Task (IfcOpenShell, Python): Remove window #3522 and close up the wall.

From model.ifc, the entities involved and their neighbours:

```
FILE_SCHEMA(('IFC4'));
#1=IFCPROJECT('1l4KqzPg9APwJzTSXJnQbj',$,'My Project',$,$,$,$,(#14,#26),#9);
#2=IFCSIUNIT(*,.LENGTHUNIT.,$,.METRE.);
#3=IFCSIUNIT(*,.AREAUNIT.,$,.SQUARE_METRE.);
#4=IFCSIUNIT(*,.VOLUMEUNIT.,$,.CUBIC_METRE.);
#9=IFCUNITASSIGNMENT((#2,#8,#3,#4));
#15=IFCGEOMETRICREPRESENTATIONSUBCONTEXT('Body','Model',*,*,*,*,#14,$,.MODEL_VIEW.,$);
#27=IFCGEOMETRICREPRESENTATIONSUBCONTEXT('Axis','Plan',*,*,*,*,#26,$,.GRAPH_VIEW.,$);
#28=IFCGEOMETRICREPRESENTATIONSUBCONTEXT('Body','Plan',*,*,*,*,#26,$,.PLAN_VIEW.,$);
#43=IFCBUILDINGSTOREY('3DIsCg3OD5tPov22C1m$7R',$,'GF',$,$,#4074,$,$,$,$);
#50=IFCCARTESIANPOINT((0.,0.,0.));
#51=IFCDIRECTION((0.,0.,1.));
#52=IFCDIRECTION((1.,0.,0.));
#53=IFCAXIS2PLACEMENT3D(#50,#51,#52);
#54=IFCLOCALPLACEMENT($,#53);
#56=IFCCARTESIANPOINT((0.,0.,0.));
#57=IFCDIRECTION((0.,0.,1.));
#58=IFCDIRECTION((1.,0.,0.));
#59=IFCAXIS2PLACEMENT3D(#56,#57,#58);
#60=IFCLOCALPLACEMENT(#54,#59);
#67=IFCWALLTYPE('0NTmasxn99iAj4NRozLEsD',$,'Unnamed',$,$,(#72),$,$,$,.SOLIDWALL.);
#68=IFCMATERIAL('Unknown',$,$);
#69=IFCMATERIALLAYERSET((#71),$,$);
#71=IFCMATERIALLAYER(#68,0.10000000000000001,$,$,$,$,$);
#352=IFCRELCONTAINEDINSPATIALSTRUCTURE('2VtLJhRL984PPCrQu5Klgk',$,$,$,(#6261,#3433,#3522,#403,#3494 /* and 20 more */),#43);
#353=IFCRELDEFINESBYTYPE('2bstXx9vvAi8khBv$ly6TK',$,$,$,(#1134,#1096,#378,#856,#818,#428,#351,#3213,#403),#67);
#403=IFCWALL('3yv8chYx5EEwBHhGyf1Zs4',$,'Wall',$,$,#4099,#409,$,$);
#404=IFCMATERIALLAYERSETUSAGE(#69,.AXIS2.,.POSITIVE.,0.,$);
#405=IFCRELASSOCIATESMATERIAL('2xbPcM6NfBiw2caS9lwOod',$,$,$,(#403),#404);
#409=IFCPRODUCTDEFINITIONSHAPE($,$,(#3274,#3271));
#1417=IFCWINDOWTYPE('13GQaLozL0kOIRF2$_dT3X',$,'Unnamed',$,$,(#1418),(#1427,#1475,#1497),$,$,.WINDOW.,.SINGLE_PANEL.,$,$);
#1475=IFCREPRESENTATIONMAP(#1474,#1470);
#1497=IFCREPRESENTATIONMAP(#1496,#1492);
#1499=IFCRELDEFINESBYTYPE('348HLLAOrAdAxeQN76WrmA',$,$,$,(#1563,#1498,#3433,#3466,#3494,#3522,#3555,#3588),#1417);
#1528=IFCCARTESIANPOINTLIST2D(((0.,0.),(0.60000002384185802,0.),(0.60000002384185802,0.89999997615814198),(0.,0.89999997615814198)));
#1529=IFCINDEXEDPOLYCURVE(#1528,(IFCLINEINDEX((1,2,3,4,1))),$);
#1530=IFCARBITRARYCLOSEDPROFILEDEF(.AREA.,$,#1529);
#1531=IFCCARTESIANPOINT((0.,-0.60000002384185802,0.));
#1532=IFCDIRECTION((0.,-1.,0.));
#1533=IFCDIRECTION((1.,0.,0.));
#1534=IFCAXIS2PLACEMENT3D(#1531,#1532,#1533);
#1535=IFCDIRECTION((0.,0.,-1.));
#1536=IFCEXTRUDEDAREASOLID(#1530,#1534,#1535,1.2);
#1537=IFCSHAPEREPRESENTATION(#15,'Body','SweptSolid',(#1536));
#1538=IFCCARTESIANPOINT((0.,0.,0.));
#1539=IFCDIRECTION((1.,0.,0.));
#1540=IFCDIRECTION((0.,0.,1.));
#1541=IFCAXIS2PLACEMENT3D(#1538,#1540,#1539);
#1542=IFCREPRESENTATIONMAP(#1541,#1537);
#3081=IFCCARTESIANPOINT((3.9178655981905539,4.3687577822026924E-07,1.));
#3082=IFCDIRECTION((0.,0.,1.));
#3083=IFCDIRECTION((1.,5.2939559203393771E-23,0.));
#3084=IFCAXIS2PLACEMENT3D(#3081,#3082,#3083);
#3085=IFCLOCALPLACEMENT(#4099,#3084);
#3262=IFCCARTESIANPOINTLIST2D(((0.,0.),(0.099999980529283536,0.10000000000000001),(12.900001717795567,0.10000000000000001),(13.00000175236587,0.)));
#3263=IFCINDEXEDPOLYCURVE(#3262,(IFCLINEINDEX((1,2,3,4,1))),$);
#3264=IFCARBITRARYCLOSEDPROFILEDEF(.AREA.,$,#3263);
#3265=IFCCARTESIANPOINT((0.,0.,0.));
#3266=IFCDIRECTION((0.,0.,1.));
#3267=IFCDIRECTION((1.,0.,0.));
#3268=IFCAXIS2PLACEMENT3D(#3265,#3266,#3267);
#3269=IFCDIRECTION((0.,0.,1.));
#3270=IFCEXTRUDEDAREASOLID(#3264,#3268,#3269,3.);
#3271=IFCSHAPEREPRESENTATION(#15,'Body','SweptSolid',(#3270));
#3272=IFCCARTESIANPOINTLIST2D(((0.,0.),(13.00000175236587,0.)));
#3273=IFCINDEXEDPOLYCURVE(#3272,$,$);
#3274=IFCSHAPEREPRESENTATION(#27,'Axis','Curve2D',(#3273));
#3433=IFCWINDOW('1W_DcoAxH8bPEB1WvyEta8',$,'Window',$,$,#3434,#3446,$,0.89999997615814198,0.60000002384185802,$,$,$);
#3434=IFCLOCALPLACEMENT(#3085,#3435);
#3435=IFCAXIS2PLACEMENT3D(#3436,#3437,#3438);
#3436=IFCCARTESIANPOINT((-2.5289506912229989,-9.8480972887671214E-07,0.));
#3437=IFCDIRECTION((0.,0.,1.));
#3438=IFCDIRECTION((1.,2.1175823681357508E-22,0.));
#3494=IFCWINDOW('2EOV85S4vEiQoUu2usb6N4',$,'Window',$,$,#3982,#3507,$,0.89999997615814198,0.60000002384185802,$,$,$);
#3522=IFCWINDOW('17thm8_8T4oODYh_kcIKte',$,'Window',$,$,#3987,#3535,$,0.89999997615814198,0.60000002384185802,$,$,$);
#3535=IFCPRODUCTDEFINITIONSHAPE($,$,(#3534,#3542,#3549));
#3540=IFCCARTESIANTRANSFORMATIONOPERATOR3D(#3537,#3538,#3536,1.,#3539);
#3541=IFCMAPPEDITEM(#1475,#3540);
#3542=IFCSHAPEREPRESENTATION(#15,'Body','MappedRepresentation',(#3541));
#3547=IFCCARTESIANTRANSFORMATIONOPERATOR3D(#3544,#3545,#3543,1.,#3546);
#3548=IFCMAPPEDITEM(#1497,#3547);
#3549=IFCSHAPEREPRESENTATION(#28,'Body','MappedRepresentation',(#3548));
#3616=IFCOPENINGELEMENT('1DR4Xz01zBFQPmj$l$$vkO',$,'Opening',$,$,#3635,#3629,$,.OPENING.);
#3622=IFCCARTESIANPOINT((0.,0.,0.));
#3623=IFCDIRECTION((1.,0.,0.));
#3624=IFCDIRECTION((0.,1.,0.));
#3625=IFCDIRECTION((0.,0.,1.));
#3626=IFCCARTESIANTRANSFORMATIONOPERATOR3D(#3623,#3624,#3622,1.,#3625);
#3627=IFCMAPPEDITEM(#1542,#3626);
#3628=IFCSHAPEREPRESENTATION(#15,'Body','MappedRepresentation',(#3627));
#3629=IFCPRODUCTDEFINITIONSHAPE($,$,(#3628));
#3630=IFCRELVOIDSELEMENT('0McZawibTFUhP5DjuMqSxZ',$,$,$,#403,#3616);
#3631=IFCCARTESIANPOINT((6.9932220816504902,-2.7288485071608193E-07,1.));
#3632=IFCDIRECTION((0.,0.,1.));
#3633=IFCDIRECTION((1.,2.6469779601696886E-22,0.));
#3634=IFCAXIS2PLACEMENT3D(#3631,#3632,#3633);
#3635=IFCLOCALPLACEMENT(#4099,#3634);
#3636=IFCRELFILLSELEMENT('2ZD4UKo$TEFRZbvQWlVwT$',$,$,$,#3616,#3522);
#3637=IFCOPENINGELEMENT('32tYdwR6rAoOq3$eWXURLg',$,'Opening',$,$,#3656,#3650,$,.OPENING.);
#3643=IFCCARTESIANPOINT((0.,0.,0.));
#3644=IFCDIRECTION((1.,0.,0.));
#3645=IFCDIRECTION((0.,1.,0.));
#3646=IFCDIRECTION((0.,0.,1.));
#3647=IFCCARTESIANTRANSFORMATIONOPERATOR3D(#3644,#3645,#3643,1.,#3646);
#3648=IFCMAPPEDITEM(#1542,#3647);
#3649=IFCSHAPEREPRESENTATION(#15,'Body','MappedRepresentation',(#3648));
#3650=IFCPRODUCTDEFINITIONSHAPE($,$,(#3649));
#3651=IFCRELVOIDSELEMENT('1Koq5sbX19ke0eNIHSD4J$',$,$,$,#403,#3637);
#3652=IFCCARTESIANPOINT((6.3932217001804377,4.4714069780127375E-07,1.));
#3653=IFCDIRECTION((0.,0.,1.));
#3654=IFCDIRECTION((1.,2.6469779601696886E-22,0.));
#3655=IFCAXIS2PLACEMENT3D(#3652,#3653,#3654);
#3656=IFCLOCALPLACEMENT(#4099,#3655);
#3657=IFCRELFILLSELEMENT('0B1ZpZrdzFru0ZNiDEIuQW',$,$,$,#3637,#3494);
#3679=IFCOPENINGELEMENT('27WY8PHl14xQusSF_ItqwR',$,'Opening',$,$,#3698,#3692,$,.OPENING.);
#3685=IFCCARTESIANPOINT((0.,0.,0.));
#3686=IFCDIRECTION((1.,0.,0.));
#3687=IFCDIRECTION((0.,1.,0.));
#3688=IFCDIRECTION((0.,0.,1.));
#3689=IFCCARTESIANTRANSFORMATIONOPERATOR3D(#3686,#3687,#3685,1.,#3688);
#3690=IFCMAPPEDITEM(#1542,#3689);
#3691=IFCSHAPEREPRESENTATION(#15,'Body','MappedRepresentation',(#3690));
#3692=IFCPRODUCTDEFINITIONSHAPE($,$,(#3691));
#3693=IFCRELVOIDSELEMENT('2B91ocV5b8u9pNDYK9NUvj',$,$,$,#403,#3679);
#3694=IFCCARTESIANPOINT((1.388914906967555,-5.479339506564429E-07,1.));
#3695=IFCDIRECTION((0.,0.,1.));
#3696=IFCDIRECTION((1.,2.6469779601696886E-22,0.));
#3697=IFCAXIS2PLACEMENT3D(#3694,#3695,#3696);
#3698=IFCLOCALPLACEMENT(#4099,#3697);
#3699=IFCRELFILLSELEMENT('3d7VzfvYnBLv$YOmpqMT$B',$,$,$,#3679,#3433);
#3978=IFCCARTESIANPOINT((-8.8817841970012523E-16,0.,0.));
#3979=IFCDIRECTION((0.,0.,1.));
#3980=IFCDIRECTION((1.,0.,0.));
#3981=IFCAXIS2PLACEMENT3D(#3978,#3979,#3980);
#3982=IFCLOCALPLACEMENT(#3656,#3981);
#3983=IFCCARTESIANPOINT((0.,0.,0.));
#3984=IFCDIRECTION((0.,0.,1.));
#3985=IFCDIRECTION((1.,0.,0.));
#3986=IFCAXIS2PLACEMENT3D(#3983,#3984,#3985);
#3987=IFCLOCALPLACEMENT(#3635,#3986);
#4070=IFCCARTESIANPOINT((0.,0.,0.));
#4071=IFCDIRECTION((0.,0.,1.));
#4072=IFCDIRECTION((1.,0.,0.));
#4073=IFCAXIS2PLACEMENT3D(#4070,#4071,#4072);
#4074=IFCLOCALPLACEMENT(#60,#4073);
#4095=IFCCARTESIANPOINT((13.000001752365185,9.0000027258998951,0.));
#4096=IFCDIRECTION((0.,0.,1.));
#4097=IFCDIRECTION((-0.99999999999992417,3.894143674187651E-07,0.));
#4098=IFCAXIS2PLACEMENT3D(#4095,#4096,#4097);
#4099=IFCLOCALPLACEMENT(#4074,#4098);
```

```python
import ifcopenshell
import ifcopenshell.api.feature
import ifcopenshell.api.root
import ifcopenshell.geom
import ifcopenshell.util.shape

model = ifcopenshell.open("model.ifc")
settings = ifcopenshell.geom.settings()


def volume(element):
    """Net volume in cubic metres, openings subtracted."""
    shape = ifcopenshell.geom.create_shape(settings, element)
    return ifcopenshell.util.shape.get_volume(shape.geometry)


window = model.by_id(3522)
opening = window.FillsVoids[0].RelatingOpeningElement
wall = opening.VoidsElements[0].RelatingBuildingElement
before = volume(wall)

ifcopenshell.api.root.remove_product(model, product=window)
ifcopenshell.api.feature.remove_feature(model, feature=opening)

after = volume(wall)

print(f"wall volume {before:.3f} -> {after:.3f} m3")

model.write("model_rev.ifc")
```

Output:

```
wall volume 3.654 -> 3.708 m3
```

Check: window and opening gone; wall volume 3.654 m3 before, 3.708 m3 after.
